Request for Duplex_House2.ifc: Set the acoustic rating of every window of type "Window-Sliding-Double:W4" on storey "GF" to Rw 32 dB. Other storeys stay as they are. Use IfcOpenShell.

First a look at what the model holds.

```python
import ifcopenshell
import ifcopenshell.util.element

model = ifcopenshell.open("Duplex_House2.ifc")
print(model.schema)
storey = next(s for s in model.by_type("IfcBuildingStorey") if s.Name == "GF")
windows = [e for e in ifcopenshell.util.element.get_decomposition(storey) if e.is_a("IfcWindow")]
seen = {}
for e in windows:
    element_type = ifcopenshell.util.element.get_type(e)
    key = (element_type.Name if element_type != e and element_type else None, ifcopenshell.util.element.get_pset(e, "Pset_WindowCommon", "AcousticRating"))
    seen[key] = seen.get(key, 0) + 1
for (name, value), count in sorted(seen.items(), key=str):
    print(count, "x", name, "|", value)
```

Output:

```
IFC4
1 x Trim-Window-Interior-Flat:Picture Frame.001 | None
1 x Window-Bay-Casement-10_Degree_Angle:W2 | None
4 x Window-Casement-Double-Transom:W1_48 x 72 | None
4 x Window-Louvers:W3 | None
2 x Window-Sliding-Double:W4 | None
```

```python
import ifcopenshell
import ifcopenshell.api.pset
import ifcopenshell.util.element

model = ifcopenshell.open("Duplex_House2.ifc")

storey = next(s for s in model.by_type("IfcBuildingStorey") if s.Name == "GF")
windows = [e for e in ifcopenshell.util.element.get_decomposition(storey) if e.is_a("IfcWindow")]

count = 0
for e in windows:
    element_type = ifcopenshell.util.element.get_type(e)
    if element_type in (None, e) or element_type.Name != "Window-Sliding-Double:W4":
        continue
    # add_pset returns the element's existing set when there is one.
    pset = ifcopenshell.api.pset.add_pset(model, product=e, name="Pset_WindowCommon")
    ifcopenshell.api.pset.edit_pset(model, pset=pset, properties={"AcousticRating": "Rw 32 dB"})
    count += 1

print(count, "windows updated")

model.write("Duplex_House2_updated.ifc")
```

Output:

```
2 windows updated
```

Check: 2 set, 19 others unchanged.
